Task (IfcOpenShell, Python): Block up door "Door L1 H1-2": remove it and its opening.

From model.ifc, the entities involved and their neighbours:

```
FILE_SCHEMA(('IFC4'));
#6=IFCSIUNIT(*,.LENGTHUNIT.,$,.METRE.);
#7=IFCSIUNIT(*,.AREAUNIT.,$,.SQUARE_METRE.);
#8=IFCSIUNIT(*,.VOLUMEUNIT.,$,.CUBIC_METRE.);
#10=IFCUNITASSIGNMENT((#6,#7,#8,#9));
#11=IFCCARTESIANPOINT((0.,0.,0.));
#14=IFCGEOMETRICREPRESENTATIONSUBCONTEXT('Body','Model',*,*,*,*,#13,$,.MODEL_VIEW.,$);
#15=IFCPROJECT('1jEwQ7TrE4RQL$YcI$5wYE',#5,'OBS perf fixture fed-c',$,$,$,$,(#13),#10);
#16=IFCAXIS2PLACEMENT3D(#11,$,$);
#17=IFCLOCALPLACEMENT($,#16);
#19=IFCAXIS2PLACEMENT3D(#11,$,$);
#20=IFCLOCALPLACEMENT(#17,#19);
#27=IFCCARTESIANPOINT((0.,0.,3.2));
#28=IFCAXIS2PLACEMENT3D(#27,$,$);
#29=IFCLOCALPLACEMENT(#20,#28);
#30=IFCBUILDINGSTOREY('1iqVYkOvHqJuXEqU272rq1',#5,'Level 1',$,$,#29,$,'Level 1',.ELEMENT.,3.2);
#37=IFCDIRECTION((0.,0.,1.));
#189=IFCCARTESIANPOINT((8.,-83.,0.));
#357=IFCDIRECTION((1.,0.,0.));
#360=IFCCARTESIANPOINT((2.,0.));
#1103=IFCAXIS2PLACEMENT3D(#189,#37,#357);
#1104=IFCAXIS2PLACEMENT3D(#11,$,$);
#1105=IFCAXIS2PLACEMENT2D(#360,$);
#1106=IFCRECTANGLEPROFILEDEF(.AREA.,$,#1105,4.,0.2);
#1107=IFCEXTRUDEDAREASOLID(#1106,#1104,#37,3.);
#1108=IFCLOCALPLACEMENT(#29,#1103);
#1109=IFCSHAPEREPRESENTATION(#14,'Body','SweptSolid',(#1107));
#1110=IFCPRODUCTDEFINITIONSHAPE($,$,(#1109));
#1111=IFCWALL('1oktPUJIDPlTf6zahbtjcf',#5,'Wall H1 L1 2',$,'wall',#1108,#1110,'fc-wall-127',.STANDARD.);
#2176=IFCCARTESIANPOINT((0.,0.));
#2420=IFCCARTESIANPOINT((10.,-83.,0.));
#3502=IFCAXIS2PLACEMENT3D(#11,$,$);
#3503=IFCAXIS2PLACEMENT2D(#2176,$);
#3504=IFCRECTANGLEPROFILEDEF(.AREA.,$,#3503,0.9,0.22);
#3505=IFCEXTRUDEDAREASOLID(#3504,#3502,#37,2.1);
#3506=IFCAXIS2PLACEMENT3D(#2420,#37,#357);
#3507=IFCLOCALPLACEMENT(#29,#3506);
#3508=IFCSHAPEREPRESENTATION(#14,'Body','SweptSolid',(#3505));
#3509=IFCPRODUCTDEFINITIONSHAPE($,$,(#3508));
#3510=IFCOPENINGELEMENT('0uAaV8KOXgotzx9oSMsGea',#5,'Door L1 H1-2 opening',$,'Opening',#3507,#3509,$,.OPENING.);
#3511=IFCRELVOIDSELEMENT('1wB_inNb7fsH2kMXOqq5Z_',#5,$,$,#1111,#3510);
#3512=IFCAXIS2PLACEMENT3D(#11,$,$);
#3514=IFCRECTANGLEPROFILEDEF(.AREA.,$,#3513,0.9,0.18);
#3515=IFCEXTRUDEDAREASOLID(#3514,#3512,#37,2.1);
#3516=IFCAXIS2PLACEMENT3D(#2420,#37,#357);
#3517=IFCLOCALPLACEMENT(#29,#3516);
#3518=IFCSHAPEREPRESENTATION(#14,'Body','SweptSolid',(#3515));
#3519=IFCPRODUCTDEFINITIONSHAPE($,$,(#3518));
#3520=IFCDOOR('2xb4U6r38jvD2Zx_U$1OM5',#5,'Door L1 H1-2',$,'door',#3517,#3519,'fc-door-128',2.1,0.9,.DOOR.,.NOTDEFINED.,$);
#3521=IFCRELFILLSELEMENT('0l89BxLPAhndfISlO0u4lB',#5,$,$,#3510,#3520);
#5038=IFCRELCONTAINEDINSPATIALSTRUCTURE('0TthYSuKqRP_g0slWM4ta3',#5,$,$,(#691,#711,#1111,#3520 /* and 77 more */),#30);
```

```python
import ifcopenshell
import ifcopenshell.api.feature
import ifcopenshell.api.root
import ifcopenshell.geom
import ifcopenshell.util.shape

model = ifcopenshell.open("model.ifc")
settings = ifcopenshell.geom.settings()


def volume(element):
    """Net volume in cubic metres, openings subtracted."""
    shape = ifcopenshell.geom.create_shape(settings, element)
    return ifcopenshell.util.shape.get_volume(shape.geometry)


door = model.by_id(3520)
opening = door.FillsVoids[0].RelatingOpeningElement
wall = opening.VoidsElements[0].RelatingBuildingElement
before = volume(wall)

ifcopenshell.api.root.remove_product(model, product=door)
ifcopenshell.api.feature.remove_feature(model, feature=opening)

after = volume(wall)

print(f"wall volume {before:.3f} -> {after:.3f} m3")

model.write("model_updated.ifc")
```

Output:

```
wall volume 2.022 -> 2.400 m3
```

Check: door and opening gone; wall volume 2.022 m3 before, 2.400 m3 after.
